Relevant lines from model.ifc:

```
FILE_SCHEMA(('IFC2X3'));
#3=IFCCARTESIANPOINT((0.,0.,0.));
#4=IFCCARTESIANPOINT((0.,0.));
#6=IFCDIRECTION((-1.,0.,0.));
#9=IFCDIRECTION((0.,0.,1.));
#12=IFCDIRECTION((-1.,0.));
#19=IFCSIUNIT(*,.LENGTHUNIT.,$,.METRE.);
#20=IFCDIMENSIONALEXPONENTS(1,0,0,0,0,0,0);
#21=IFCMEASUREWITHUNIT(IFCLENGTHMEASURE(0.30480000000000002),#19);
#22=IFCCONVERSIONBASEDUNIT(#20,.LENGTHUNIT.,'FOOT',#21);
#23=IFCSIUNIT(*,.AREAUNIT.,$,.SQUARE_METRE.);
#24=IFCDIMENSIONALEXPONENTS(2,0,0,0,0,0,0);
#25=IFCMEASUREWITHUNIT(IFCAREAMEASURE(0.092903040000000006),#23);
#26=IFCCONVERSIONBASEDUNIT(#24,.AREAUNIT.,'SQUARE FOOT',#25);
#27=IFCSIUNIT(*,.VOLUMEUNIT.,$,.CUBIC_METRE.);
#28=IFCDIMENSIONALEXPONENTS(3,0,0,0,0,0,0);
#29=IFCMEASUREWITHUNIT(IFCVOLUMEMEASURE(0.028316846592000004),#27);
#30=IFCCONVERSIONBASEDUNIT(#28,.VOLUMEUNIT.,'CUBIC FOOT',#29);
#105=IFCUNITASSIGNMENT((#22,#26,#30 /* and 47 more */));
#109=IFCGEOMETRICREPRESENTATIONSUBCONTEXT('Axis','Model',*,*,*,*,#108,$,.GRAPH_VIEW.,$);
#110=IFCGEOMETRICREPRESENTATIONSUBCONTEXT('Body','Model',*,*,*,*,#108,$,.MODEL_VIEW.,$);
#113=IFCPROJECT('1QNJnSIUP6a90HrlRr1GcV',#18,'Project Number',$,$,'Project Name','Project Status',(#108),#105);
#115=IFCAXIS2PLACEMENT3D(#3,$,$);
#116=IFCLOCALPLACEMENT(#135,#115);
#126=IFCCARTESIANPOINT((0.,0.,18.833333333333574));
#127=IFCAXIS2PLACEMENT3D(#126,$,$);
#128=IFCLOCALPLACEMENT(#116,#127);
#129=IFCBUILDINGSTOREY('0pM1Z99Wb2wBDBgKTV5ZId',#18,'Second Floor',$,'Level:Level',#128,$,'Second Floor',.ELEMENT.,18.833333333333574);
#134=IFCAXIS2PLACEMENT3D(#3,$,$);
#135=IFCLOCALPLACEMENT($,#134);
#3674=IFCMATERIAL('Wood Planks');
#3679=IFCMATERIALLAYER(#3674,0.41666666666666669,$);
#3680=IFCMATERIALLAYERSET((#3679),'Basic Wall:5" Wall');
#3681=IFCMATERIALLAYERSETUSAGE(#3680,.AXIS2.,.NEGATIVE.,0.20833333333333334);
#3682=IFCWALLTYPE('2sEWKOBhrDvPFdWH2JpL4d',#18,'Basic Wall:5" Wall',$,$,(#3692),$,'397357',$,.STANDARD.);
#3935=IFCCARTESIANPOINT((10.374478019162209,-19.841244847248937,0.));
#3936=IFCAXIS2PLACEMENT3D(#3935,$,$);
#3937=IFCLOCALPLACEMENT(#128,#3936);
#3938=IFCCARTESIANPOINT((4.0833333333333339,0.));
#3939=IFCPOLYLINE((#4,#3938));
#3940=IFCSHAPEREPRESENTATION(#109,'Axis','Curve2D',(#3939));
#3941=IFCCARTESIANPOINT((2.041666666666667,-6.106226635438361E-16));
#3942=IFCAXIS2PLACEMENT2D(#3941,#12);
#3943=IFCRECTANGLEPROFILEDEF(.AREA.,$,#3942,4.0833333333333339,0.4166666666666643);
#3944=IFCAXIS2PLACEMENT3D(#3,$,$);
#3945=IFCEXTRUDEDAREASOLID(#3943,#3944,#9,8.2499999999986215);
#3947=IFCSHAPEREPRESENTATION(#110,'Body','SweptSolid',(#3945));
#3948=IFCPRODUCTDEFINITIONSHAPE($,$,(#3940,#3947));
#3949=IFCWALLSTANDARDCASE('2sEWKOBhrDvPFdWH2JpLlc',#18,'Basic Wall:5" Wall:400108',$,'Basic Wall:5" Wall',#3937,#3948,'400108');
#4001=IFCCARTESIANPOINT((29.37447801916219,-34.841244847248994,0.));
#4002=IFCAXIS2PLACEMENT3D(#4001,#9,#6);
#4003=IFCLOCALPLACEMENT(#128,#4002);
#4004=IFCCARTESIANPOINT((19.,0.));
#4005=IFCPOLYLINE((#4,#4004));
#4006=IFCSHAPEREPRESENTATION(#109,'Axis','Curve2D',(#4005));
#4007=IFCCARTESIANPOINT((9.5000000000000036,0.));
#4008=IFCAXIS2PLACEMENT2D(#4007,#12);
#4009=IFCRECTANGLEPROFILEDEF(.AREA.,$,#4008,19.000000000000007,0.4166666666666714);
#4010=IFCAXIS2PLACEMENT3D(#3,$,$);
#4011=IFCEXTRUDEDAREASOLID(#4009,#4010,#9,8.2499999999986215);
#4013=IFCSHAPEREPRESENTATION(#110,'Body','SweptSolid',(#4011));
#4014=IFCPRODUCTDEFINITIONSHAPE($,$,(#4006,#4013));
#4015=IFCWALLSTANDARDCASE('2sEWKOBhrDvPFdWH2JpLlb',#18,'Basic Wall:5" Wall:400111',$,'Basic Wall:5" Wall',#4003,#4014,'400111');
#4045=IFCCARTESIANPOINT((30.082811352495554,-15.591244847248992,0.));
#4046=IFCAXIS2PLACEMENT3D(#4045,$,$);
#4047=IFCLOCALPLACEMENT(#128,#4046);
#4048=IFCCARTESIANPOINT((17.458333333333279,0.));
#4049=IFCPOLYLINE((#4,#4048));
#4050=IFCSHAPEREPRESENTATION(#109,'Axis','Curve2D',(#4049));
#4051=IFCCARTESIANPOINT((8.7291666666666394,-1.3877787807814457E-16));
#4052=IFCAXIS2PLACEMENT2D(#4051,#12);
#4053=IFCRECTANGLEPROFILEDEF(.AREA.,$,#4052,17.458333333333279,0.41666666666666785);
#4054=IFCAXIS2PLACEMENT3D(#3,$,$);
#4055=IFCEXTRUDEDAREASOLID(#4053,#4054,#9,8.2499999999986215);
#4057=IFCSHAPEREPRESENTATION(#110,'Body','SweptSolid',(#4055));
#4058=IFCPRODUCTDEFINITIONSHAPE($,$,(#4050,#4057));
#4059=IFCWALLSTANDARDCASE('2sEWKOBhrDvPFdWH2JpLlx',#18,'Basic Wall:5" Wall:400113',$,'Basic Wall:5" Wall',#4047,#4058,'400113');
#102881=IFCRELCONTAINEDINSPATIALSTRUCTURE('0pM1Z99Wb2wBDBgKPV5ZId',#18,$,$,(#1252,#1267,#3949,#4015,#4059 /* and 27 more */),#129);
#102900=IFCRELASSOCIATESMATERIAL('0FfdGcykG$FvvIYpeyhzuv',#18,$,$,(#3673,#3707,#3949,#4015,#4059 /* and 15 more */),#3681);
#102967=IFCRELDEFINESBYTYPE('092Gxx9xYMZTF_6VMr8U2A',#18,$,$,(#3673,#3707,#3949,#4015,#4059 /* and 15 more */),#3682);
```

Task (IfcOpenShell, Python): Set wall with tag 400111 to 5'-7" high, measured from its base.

```python
import ifcopenshell
import ifcopenshell.geom
import ifcopenshell.util.representation
import ifcopenshell.util.shape
import ifcopenshell.util.unit

model = ifcopenshell.open("model.ifc")
unit_scale = ifcopenshell.util.unit.calculate_unit_scale(model)
settings = ifcopenshell.geom.settings()


def volume(element):
    """Net volume in cubic metres, openings subtracted."""
    shape = ifcopenshell.geom.create_shape(settings, element)
    return ifcopenshell.util.shape.get_volume(shape.geometry)


wall = model.by_id(4015)
before = volume(wall)

body = ifcopenshell.util.representation.get_representation(wall, "Model", "Body")
solid = body.Items[0]
old_height = solid.Depth
solid.Depth = 67 * 0.0254 / unit_scale
after = volume(wall)

print(f"height {old_height:g} -> {solid.Depth:g}, volume {before:.3f} -> {after:.3f} m3")

model.write("model_rev.ifc")
```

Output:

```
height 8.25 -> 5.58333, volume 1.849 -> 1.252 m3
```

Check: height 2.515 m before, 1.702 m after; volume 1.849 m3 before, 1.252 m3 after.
